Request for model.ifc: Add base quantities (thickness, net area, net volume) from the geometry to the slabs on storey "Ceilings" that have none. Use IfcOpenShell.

First a look at what the model holds.

```python
import ifcopenshell
import ifcopenshell.util.element
import ifcopenshell.util.unit

model = ifcopenshell.open("model.ifc")
print(model.schema)
for unit_type in ("LENGTHUNIT", "AREAUNIT", "VOLUMEUNIT"):
    print(unit_type, ifcopenshell.util.unit.calculate_unit_scale(model, unit_type))
storey = next(s for s in model.by_type("IfcBuildingStorey") if s.Name == "Ceilings")
slabs = [e for e in ifcopenshell.util.element.get_decomposition(storey) if e.is_a("IfcSlab")]
for e in sorted(slabs, key=lambda e: e.id()):
    print(e.id(), e.is_a(), e.Name, list(ifcopenshell.util.element.get_psets(e, qtos_only=True)), sep=" | ")
```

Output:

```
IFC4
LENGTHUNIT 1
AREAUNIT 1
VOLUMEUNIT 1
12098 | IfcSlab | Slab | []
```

```python
import ifcopenshell
import ifcopenshell.api.pset
import ifcopenshell.geom
import ifcopenshell.util.element
import ifcopenshell.util.shape
import ifcopenshell.util.unit

model = ifcopenshell.open("model.ifc")
unit_scale = ifcopenshell.util.unit.calculate_unit_scale(model)
area_scale = ifcopenshell.util.unit.calculate_unit_scale(model, "AREAUNIT")
volume_scale = ifcopenshell.util.unit.calculate_unit_scale(model, "VOLUMEUNIT")
settings = ifcopenshell.geom.settings()

storey = next(s for s in model.by_type("IfcBuildingStorey") if s.Name == "Ceilings")
slabs = [e for e in ifcopenshell.util.element.get_decomposition(storey) if e.is_a("IfcSlab")]

for e in sorted(slabs, key=lambda e: e.id()):
    if ifcopenshell.util.element.get_psets(e, qtos_only=True, should_inherit=False):
        continue
    # Geometry comes back in metres, in the element's own axes.
    shape = ifcopenshell.geom.create_shape(settings, e)
    values = {
        "Width": ifcopenshell.util.shape.get_z(shape.geometry) / unit_scale,
        "NetArea": ifcopenshell.util.shape.get_footprint_area(shape.geometry) / area_scale,
        "NetVolume": ifcopenshell.util.shape.get_volume(shape.geometry) / volume_scale,
    }
    qto = ifcopenshell.api.pset.add_qto(model, product=e, name="Qto_SlabBaseQuantities")
    ifcopenshell.api.pset.edit_qto(model, qto=qto, properties=values)
    print(e.id(), {k: round(v, 3) for k, v in values.items()})

model.write("model-out.ifc")
```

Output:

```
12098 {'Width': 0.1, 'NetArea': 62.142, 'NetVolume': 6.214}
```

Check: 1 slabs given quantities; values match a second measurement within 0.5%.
